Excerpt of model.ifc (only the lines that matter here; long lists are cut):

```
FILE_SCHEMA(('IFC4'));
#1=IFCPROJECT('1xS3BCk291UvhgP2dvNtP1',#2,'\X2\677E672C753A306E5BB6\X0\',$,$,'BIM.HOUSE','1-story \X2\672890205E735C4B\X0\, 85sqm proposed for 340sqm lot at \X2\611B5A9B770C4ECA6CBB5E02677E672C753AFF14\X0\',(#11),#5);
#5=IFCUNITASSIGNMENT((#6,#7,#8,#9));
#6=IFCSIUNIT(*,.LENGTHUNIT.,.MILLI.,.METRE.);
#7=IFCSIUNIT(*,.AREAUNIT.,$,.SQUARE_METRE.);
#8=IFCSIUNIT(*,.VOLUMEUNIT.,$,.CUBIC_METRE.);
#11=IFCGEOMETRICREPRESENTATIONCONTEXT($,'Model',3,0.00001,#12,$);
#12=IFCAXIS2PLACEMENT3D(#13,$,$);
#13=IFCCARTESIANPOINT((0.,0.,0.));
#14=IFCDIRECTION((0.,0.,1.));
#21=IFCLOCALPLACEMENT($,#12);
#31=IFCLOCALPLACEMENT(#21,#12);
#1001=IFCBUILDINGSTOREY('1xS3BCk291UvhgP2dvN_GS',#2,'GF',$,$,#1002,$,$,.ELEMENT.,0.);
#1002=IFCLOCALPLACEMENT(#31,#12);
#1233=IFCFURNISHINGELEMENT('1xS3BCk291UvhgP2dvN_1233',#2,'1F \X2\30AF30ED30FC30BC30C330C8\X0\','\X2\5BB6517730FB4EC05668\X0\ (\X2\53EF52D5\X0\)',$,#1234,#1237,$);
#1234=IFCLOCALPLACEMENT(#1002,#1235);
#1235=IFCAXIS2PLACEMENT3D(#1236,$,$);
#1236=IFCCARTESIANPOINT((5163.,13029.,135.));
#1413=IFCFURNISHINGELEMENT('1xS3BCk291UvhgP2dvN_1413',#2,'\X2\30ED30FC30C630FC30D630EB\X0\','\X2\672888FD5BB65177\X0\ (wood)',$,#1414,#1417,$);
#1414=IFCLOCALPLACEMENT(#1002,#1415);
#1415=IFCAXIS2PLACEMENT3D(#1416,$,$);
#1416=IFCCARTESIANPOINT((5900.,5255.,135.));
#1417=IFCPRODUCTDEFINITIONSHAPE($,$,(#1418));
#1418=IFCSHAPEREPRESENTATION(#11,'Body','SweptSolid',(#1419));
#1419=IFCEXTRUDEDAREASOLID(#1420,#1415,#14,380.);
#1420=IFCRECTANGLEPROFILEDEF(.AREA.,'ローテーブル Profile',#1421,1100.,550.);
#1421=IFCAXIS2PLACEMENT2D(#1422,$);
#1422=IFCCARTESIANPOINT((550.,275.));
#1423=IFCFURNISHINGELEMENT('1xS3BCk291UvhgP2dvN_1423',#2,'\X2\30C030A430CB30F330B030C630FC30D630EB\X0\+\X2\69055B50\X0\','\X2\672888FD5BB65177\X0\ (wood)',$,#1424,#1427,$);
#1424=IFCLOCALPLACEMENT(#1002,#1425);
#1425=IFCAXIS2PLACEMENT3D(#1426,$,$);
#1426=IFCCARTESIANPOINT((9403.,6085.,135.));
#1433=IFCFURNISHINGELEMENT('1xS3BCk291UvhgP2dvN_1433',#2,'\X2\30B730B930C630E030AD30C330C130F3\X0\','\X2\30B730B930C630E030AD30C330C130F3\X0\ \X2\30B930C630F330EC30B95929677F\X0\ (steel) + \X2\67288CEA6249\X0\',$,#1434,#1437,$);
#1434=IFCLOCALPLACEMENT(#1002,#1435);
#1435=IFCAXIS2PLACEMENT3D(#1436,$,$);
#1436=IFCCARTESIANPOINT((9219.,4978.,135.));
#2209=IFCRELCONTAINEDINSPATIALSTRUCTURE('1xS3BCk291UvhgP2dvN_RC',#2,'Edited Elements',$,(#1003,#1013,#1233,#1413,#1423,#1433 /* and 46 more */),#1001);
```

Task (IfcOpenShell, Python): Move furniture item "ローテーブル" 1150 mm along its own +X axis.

```python
import ifcopenshell
import ifcopenshell.api.geometry
import ifcopenshell.util.placement
import ifcopenshell.util.unit

model = ifcopenshell.open("model.ifc")
unit_scale = ifcopenshell.util.unit.calculate_unit_scale(model)

item = model.by_guid("1xS3BCk291UvhgP2dvN_1413")
matrix = ifcopenshell.util.placement.get_local_placement(item.ObjectPlacement)
matrix[:3, 3] += matrix[:3, 0] * 1.15 / unit_scale
ifcopenshell.api.geometry.edit_object_placement(model, product=item, matrix=matrix, is_si=False)

print(ifcopenshell.util.placement.get_local_placement(item.ObjectPlacement).round(3) + 0.0)

model.write("model-out.ifc")
```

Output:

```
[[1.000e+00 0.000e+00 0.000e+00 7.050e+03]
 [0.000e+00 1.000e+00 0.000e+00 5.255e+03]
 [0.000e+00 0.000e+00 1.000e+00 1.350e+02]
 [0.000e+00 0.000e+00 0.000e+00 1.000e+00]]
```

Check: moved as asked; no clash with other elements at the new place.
